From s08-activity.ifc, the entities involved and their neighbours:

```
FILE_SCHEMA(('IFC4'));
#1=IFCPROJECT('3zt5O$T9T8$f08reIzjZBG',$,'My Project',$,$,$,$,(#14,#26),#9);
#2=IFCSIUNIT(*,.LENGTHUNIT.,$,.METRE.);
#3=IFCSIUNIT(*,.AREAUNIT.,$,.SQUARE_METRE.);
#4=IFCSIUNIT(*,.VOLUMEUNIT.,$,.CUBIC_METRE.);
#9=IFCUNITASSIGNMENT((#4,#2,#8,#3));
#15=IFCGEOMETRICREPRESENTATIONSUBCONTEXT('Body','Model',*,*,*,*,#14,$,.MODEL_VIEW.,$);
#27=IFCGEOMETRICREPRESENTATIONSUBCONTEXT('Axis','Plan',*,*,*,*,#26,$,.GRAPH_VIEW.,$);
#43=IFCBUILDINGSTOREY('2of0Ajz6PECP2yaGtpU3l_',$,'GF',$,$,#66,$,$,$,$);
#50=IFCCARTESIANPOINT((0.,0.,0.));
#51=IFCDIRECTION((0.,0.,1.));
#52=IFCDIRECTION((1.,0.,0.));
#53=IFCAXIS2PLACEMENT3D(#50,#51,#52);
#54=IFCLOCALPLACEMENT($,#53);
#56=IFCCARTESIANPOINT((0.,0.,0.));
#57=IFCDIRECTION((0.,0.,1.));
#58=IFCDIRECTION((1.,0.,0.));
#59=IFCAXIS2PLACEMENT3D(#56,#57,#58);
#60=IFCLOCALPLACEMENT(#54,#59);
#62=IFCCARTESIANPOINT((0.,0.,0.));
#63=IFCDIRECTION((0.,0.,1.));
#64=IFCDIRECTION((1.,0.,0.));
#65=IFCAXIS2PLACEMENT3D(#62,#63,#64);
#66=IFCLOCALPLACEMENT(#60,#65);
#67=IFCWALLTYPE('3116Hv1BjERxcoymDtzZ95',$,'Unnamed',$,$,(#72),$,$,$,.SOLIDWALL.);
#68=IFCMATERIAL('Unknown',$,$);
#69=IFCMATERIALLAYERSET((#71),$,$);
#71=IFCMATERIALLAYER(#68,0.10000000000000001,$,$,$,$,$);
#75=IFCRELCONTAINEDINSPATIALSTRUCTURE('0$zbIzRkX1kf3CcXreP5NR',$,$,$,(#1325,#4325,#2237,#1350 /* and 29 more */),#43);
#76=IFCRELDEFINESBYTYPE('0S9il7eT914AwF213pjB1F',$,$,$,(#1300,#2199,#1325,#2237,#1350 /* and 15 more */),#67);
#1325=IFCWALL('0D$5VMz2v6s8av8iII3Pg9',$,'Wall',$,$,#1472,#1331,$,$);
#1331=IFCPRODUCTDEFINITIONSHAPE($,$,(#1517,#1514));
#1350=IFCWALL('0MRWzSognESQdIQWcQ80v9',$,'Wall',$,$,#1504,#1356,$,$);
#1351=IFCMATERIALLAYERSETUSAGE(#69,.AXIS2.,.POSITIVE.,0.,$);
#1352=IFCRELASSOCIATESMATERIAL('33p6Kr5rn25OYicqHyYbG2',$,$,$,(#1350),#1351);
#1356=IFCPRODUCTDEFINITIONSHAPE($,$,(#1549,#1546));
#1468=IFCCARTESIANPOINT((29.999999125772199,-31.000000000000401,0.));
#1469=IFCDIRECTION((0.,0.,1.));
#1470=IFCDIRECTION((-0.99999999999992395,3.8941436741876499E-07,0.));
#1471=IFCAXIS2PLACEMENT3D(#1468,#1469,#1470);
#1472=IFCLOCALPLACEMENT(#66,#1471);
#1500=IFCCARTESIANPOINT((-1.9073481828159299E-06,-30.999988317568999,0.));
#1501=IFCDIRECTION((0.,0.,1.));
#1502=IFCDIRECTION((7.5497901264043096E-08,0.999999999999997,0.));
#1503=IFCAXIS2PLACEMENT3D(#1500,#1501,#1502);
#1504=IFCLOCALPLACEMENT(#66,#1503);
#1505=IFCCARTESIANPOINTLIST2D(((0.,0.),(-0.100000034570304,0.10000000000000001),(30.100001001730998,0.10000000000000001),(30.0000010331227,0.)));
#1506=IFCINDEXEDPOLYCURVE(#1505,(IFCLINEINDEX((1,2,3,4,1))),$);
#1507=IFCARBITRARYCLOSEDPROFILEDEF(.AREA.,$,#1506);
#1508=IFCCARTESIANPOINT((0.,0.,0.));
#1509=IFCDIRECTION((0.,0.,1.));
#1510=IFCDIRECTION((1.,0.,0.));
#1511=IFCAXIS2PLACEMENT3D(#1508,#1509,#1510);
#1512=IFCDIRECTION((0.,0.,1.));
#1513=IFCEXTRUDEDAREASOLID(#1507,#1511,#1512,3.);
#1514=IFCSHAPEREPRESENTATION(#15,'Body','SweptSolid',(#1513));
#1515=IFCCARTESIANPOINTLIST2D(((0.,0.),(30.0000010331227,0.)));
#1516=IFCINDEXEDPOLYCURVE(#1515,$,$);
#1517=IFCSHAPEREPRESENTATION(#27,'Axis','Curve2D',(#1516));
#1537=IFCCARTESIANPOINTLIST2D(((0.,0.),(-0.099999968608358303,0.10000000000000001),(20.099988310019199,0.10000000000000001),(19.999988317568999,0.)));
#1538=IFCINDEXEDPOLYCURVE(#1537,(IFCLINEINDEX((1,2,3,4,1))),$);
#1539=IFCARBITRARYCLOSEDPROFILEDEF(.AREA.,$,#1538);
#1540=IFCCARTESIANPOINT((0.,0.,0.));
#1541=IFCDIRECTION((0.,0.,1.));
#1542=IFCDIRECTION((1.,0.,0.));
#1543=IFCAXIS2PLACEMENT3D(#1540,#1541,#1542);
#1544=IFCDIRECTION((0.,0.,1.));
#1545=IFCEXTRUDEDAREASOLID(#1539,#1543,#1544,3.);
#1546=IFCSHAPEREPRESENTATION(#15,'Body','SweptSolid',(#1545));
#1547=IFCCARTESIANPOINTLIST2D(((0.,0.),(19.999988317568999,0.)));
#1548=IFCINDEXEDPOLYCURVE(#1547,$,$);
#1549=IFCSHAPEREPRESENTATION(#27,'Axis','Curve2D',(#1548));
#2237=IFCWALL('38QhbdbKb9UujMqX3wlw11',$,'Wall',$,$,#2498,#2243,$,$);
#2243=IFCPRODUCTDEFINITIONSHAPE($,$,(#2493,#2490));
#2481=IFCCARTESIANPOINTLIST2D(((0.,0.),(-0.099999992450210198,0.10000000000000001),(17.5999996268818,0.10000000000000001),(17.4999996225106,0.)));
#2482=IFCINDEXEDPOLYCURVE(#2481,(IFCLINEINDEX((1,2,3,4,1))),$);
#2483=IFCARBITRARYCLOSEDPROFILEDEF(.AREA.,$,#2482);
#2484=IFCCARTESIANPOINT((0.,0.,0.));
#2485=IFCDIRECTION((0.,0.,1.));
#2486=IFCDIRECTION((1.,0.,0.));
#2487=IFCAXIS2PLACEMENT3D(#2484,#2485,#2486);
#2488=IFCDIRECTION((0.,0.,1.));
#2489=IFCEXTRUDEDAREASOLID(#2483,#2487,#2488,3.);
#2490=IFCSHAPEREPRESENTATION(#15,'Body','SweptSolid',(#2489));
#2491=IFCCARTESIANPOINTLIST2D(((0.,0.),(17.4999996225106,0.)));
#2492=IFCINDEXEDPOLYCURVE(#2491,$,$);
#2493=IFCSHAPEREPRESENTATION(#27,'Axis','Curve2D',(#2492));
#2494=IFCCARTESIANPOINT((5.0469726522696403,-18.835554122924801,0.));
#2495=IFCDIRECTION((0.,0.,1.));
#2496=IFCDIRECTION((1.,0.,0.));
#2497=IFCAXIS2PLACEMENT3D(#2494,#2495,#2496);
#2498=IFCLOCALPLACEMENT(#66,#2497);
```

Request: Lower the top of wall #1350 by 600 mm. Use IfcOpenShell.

```python
import ifcopenshell
import ifcopenshell.geom
import ifcopenshell.util.representation
import ifcopenshell.util.shape
import ifcopenshell.util.unit

model = ifcopenshell.open("s08-activity.ifc")
unit_scale = ifcopenshell.util.unit.calculate_unit_scale(model)
settings = ifcopenshell.geom.settings()


def volume(element):
    """Net volume in cubic metres, openings subtracted."""
    shape = ifcopenshell.geom.create_shape(settings, element)
    return ifcopenshell.util.shape.get_volume(shape.geometry)


wall = model.by_guid("0MRWzSognESQdIQWcQ80v9")
before = volume(wall)

body = ifcopenshell.util.representation.get_representation(wall, "Model", "Body")
solid = body.Items[0]
old_height = solid.Depth
solid.Depth -= 0.6 / unit_scale
after = volume(wall)

print(f"height {old_height:g} -> {solid.Depth:g}, volume {before:.3f} -> {after:.3f} m3")

model.write("s08-activity_edited.ifc")
```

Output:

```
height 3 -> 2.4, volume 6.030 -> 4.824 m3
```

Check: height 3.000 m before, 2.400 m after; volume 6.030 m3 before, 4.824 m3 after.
